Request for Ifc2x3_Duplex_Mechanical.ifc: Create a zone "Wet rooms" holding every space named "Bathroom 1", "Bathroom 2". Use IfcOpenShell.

First a look at what the model holds.

```python
import ifcopenshell

model = ifcopenshell.open("Ifc2x3_Duplex_Mechanical.ifc")
print(model.schema)
seen = {}
for space in model.by_type("IfcSpace"):
    seen[space.LongName] = seen.get(space.LongName, 0) + 1
for name, count in sorted(seen.items(), key=str):
    print(count, "x", name)
print("zones:", [z.Name for z in model.by_type("IfcZone")][:20])
```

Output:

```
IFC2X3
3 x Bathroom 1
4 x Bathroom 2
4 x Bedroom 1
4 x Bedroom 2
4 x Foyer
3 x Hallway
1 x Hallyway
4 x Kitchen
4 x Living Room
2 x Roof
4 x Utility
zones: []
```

```python
import ifcopenshell
import ifcopenshell.api.group
import ifcopenshell.api.root

model = ifcopenshell.open("Ifc2x3_Duplex_Mechanical.ifc")

names = {"Bathroom 1", "Bathroom 2"}
spaces = [s for s in model.by_type("IfcSpace") if s.LongName in names]

zone = ifcopenshell.api.root.create_entity(model, ifc_class="IfcZone", name="Wet rooms")
ifcopenshell.api.group.assign_group(model, products=spaces, group=zone)
print(len(spaces), "spaces in", zone.Name)

model.write("Ifc2x3_Duplex_Mechanical_v2.ifc")
```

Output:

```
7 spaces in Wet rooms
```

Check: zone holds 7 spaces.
